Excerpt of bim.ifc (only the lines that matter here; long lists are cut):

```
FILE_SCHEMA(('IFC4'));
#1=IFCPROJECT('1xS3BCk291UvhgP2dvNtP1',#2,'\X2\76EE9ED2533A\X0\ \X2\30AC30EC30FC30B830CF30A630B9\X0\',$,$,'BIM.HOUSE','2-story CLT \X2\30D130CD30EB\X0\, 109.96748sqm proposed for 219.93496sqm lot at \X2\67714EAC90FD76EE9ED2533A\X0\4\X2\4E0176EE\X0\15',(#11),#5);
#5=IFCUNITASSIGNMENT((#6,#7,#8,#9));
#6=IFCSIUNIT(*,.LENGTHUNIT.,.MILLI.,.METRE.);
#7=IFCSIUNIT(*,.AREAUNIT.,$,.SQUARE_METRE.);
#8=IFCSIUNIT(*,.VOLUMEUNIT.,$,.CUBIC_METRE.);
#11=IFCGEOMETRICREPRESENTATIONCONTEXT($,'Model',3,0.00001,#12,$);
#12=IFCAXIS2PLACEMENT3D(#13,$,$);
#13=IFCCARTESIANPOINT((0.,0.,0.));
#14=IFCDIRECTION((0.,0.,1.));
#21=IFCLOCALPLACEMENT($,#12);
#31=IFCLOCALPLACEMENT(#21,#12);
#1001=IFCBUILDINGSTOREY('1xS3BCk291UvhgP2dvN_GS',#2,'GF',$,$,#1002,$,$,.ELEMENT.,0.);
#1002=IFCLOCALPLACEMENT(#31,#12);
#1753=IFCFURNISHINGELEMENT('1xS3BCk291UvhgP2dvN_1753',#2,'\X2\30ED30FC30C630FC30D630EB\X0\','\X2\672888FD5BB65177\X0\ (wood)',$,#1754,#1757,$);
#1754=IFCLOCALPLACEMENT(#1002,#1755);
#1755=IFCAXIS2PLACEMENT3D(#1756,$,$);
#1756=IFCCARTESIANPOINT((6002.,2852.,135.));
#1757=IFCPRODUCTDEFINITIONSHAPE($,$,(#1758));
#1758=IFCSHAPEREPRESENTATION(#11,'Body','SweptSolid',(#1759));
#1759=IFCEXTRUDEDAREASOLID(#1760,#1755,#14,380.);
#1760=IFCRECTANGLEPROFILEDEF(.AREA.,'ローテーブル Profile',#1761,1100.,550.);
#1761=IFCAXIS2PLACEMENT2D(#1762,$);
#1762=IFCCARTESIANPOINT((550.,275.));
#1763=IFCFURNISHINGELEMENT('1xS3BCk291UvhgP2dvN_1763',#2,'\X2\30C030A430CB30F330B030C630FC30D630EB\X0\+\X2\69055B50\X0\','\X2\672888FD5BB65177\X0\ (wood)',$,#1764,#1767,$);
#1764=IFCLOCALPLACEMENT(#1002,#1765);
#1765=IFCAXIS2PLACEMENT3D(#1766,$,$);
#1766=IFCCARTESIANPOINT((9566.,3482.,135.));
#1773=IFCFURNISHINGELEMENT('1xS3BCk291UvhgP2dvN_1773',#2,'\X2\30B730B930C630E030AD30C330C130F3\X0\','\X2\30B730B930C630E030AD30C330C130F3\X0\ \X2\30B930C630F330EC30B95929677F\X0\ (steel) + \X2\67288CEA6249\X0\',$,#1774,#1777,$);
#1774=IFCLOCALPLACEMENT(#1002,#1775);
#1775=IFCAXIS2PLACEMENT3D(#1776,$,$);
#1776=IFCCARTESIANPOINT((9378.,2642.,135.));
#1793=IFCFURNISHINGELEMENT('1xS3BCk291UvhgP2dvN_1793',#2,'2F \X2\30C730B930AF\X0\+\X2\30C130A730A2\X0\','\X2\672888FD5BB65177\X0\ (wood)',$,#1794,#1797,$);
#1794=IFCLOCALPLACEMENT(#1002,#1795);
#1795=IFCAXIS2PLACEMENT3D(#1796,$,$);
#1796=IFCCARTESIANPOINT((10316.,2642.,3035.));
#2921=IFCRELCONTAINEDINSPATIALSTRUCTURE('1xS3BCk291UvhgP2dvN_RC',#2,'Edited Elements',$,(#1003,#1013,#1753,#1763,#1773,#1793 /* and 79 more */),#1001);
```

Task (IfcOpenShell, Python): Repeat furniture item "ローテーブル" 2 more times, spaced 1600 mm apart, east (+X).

```python
import numpy as np
import ifcopenshell
import ifcopenshell.api.geometry
import ifcopenshell.api.root
import ifcopenshell.util.element
import ifcopenshell.util.placement

model = ifcopenshell.open("bim.ifc")


def reuse_history(source, copy):
    """copy_class also copies each property set's owner history, people and application; keep the originals."""
    for rel in copy.IsDefinedBy:
        if rel.is_a("IfcRelDefinesByProperties") and (history := rel.RelatingPropertyDefinition.OwnerHistory):
            rel.RelatingPropertyDefinition.OwnerHistory = source.OwnerHistory
            ifcopenshell.util.element.remove_deep2(model, history)


source = model.by_guid("1xS3BCk291UvhgP2dvN_1753")
base = ifcopenshell.util.placement.get_local_placement(source.ObjectPlacement)
step = np.array([1.0, 0.0, 0.0]) * 1600.0

for i in range(1, 3):
    copy = ifcopenshell.api.root.copy_class(model, product=source)
    copy.Representation = ifcopenshell.util.element.copy_deep(
        model, source.Representation, exclude=["IfcGeometricRepresentationContext", "IfcRepresentationMap"]
    )
    reuse_history(source, copy)
    matrix = base.copy()
    matrix[:3, 3] += i * step
    print("added at", matrix[:3, 3].round(3) + 0.0)
    ifcopenshell.api.geometry.edit_object_placement(model, product=copy, matrix=matrix, is_si=False)

model.write("bim_edited.ifc")
```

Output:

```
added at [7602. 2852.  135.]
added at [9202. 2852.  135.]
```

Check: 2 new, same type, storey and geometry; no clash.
